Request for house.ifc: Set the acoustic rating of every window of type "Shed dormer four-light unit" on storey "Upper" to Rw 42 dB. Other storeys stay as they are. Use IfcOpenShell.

First a look at what the model holds.

```python
import ifcopenshell
import ifcopenshell.util.element

model = ifcopenshell.open("house.ifc")
print(model.schema)
storey = next(s for s in model.by_type("IfcBuildingStorey") if s.Name == "Upper")
windows = [e for e in ifcopenshell.util.element.get_decomposition(storey) if e.is_a("IfcWindow")]
seen = {}
for e in windows:
    element_type = ifcopenshell.util.element.get_type(e)
    key = (element_type.Name if element_type != e and element_type else None, ifcopenshell.util.element.get_pset(e, "Pset_WindowCommon", "AcousticRating"))
    seen[key] = seen.get(key, 0) + 1
for (name, value), count in sorted(seen.items(), key=str):
    print(count, "x", name, "|", value)
```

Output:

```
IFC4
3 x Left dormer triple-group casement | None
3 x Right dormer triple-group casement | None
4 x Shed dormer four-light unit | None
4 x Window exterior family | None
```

```python
import ifcopenshell
import ifcopenshell.api.pset
import ifcopenshell.util.element

model = ifcopenshell.open("house.ifc")

storey = next(s for s in model.by_type("IfcBuildingStorey") if s.Name == "Upper")
windows = [e for e in ifcopenshell.util.element.get_decomposition(storey) if e.is_a("IfcWindow")]

count = 0
for e in windows:
    element_type = ifcopenshell.util.element.get_type(e)
    if element_type in (None, e) or element_type.Name != "Shed dormer four-light unit":
        continue
    # add_pset returns the element's existing set when there is one.
    pset = ifcopenshell.api.pset.add_pset(model, product=e, name="Pset_WindowCommon")
    ifcopenshell.api.pset.edit_pset(model, pset=pset, properties={"AcousticRating": "Rw 42 dB"})
    count += 1

print(count, "windows updated")

model.write("house_updated.ifc")
```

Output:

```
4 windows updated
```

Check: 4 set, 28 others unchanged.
